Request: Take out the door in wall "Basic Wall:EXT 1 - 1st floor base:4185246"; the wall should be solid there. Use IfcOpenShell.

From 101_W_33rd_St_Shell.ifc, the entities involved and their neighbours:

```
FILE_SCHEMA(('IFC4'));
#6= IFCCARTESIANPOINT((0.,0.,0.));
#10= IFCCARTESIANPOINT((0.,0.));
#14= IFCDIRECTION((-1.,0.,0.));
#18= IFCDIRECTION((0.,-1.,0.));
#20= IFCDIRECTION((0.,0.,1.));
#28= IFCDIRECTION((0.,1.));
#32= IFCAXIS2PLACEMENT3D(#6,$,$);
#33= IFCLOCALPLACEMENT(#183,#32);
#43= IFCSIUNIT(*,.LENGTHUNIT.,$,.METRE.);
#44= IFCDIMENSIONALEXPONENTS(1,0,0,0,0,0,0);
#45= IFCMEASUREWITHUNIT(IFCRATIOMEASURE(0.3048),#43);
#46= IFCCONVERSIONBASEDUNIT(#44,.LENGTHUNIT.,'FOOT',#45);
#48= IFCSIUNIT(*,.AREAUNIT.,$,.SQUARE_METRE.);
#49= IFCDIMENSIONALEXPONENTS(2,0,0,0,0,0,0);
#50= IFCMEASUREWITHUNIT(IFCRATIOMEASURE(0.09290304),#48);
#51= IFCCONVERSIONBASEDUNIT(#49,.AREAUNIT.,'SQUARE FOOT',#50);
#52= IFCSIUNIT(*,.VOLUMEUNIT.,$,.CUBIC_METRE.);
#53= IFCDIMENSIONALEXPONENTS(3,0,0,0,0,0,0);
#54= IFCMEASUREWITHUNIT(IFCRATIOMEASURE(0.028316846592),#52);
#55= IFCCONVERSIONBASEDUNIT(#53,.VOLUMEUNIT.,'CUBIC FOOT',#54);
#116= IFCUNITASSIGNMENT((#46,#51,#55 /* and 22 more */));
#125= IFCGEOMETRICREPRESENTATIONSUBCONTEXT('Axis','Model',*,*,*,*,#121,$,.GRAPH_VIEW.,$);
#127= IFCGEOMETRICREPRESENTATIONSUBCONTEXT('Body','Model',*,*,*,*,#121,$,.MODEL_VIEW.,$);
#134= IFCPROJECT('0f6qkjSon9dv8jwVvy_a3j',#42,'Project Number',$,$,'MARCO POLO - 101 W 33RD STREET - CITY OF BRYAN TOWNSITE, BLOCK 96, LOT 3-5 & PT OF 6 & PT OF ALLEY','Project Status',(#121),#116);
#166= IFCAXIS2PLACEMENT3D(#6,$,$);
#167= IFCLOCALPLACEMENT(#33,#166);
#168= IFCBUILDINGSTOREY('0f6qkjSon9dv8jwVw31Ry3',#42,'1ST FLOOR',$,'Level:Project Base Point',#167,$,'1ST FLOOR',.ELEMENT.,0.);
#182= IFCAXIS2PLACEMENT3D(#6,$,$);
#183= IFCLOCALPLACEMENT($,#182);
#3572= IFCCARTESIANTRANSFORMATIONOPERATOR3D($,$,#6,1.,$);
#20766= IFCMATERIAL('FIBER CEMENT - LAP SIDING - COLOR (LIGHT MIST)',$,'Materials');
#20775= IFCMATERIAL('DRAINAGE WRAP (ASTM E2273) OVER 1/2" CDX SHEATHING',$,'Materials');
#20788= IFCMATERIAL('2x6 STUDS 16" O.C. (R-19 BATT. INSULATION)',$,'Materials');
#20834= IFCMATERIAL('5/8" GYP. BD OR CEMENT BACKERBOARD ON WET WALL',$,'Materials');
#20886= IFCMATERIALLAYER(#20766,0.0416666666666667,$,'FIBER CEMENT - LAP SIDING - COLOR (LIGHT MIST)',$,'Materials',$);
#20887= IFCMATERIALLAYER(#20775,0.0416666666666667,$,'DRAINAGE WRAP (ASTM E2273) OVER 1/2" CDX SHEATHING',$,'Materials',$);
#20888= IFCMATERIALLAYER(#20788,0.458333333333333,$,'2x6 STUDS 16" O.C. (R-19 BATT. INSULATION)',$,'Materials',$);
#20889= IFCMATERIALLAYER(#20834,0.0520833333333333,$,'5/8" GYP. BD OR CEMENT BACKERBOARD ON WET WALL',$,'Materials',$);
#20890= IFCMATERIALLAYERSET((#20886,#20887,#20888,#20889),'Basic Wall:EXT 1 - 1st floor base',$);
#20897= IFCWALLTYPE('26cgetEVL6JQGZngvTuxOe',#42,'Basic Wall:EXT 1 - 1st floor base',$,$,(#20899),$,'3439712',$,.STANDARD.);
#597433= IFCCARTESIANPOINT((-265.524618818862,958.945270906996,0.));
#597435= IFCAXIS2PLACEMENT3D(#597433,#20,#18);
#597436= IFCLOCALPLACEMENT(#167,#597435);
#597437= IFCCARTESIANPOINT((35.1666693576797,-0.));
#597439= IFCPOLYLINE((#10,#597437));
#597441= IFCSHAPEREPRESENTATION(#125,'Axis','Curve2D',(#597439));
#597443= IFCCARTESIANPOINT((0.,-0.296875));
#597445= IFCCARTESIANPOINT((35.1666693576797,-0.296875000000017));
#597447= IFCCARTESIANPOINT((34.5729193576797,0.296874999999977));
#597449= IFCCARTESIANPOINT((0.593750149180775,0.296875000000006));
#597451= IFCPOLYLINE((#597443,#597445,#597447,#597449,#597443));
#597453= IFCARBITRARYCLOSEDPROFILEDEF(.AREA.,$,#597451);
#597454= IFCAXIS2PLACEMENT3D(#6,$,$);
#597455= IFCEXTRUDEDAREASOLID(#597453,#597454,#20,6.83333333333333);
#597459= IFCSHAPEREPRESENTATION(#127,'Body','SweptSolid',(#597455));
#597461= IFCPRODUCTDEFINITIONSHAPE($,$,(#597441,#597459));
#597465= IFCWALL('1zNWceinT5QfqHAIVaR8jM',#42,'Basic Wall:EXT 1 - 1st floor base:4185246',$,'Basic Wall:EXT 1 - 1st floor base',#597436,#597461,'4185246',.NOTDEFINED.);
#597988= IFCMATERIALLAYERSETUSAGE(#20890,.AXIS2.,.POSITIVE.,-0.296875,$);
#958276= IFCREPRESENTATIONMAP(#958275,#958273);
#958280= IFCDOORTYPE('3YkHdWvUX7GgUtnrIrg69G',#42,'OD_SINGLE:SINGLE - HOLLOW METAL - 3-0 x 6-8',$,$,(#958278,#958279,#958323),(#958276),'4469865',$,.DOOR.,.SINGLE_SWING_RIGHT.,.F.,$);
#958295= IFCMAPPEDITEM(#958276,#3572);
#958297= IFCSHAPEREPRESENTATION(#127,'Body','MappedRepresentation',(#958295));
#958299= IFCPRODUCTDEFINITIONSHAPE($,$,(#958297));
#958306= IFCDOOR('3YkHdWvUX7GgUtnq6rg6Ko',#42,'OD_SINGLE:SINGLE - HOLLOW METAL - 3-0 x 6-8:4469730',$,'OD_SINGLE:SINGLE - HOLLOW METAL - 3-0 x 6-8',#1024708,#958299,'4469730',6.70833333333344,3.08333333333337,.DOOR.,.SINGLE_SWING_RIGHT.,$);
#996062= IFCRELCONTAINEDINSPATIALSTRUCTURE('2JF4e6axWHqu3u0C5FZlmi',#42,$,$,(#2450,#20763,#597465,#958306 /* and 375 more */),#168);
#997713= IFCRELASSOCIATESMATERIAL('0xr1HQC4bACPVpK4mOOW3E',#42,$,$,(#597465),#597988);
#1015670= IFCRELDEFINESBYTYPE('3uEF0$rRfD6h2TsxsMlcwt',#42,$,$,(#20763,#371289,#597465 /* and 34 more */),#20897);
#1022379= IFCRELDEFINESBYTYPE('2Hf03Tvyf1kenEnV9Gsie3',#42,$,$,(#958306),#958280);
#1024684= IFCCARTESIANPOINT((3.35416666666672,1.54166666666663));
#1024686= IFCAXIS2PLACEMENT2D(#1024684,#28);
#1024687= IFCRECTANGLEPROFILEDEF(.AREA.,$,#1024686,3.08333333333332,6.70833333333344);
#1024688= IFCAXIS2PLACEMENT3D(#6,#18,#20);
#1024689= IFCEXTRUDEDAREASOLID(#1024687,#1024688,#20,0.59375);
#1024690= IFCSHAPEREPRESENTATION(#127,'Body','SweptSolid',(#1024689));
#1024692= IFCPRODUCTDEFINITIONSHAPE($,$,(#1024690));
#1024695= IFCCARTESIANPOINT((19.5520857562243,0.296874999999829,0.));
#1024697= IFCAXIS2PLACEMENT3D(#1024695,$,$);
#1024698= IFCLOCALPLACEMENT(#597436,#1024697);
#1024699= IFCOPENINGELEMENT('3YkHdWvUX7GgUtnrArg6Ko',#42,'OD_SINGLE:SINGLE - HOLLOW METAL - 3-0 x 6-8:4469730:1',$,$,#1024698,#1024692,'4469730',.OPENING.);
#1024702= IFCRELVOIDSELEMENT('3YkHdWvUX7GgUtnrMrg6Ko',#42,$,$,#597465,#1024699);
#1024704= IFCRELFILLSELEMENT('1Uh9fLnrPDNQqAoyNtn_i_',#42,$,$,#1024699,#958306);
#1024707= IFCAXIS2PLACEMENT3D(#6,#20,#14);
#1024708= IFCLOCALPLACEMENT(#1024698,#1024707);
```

```python
import ifcopenshell
import ifcopenshell.api.feature
import ifcopenshell.api.root
import ifcopenshell.geom
import ifcopenshell.util.shape

model = ifcopenshell.open("101_W_33rd_St_Shell.ifc")
settings = ifcopenshell.geom.settings()


def volume(element):
    """Net volume in cubic metres, openings subtracted."""
    shape = ifcopenshell.geom.create_shape(settings, element)
    return ifcopenshell.util.shape.get_volume(shape.geometry)


door = model.by_id(958306)
opening = door.FillsVoids[0].RelatingOpeningElement
wall = opening.VoidsElements[0].RelatingBuildingElement
before = volume(wall)

ifcopenshell.api.root.remove_product(model, product=door)
ifcopenshell.api.feature.remove_feature(model, feature=opening)

after = volume(wall)

print(f"wall volume {before:.3f} -> {after:.3f} m3")

model.write("101_W_33rd_St_Shell_updated.ifc")
```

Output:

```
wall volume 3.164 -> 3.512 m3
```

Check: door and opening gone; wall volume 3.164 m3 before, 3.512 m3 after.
